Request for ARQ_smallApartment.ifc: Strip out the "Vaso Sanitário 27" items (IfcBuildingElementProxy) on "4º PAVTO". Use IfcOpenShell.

First a look at what the model holds.

```python
import ifcopenshell
import ifcopenshell.util.element

model = ifcopenshell.open("ARQ_smallApartment.ifc")
print(model.schema)
storey = next(s for s in model.by_type("IfcBuildingStorey") if s.Name == "4º PAVTO")
proxies = [e for e in ifcopenshell.util.element.get_decomposition(storey) if e.is_a("IfcBuildingElementProxy")]
seen = {}
for e in proxies:
    element_type = ifcopenshell.util.element.get_type(e)
    name = element_type.Name if element_type not in (None, e) else None
    seen[name] = seen.get(name, 0) + 1
for name, count in sorted(seen.items(), key=str):
    print(count, "x", name)
```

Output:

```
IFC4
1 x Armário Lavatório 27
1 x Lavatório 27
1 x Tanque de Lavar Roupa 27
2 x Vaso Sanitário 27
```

```python
import ifcopenshell
import ifcopenshell.api.root
import ifcopenshell.util.element

model = ifcopenshell.open("ARQ_smallApartment.ifc")

storey = next(s for s in model.by_type("IfcBuildingStorey") if s.Name == "4º PAVTO")
proxies = [e for e in ifcopenshell.util.element.get_decomposition(storey) if e.is_a("IfcBuildingElementProxy")]
targets = [e for e in proxies if (t := ifcopenshell.util.element.get_type(e)) not in (None, e) and t.Name == "Vaso Sanitário 27"]

for e in targets:
    ifcopenshell.api.root.remove_product(model, product=e)
print(len(targets), "removed")

model.write("ARQ_smallApartment_rev.ifc")
```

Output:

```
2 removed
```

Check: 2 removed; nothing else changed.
